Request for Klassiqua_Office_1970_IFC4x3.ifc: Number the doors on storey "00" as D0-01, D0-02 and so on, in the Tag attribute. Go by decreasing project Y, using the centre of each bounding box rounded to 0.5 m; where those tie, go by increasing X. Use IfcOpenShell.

First a look at what the model holds.

```python
import ifcopenshell
import ifcopenshell.util.element
import ifcopenshell.util.placement

model = ifcopenshell.open("Klassiqua_Office_1970_IFC4x3.ifc")
print(model.schema)
storey = next(s for s in model.by_type("IfcBuildingStorey") if s.Name == "00")
doors = [e for e in ifcopenshell.util.element.get_decomposition(storey) if e.is_a("IfcDoor")]
for e in sorted(doors, key=lambda e: e.id()):
    origin = ifcopenshell.util.placement.get_local_placement(e.ObjectPlacement)[:3, 3]
    print(e.id(), e.Tag, e.Name, origin.round(2) + 0.0, sep=" | ")
```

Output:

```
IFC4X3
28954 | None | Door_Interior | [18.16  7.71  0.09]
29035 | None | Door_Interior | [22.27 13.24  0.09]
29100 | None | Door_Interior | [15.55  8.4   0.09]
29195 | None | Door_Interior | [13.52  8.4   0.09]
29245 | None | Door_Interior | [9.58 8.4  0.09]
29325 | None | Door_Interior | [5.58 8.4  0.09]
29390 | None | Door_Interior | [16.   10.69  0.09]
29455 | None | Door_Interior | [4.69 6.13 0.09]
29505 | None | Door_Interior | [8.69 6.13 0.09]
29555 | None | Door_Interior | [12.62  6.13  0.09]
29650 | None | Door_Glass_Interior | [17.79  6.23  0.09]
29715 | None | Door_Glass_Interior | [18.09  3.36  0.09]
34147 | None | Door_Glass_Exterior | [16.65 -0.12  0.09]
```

```python
import ifcopenshell
import ifcopenshell.geom
import ifcopenshell.util.element
import ifcopenshell.util.shape

model = ifcopenshell.open("Klassiqua_Office_1970_IFC4x3.ifc")
settings = ifcopenshell.geom.settings()
settings.set("use-world-coords", True)


def centre(element):
    shape = ifcopenshell.geom.create_shape(settings, element)
    return ifcopenshell.util.shape.get_bbox_centroid(shape.geometry)


storey = next(s for s in model.by_type("IfcBuildingStorey") if s.Name == "00")
doors = [e for e in ifcopenshell.util.element.get_decomposition(storey) if e.is_a("IfcDoor")]

# Insertion points can sit at a corner or the storey origin, so sort by the geometry (in metres).
centres = {e: centre(e) for e in doors}
doors.sort(key=lambda e: (-round(centres[e][1] / 0.5), centres[e][0]))

for i, e in enumerate(doors, start=1):
    number = f"D0-{i:02d}"
    e.Tag = number
    print(e.id(), number)

model.write("Klassiqua_Office_1970_IFC4x3_edited.ifc")
```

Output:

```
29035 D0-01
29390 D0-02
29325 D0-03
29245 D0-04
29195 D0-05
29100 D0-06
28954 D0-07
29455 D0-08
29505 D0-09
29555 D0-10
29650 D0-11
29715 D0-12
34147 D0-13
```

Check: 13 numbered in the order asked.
